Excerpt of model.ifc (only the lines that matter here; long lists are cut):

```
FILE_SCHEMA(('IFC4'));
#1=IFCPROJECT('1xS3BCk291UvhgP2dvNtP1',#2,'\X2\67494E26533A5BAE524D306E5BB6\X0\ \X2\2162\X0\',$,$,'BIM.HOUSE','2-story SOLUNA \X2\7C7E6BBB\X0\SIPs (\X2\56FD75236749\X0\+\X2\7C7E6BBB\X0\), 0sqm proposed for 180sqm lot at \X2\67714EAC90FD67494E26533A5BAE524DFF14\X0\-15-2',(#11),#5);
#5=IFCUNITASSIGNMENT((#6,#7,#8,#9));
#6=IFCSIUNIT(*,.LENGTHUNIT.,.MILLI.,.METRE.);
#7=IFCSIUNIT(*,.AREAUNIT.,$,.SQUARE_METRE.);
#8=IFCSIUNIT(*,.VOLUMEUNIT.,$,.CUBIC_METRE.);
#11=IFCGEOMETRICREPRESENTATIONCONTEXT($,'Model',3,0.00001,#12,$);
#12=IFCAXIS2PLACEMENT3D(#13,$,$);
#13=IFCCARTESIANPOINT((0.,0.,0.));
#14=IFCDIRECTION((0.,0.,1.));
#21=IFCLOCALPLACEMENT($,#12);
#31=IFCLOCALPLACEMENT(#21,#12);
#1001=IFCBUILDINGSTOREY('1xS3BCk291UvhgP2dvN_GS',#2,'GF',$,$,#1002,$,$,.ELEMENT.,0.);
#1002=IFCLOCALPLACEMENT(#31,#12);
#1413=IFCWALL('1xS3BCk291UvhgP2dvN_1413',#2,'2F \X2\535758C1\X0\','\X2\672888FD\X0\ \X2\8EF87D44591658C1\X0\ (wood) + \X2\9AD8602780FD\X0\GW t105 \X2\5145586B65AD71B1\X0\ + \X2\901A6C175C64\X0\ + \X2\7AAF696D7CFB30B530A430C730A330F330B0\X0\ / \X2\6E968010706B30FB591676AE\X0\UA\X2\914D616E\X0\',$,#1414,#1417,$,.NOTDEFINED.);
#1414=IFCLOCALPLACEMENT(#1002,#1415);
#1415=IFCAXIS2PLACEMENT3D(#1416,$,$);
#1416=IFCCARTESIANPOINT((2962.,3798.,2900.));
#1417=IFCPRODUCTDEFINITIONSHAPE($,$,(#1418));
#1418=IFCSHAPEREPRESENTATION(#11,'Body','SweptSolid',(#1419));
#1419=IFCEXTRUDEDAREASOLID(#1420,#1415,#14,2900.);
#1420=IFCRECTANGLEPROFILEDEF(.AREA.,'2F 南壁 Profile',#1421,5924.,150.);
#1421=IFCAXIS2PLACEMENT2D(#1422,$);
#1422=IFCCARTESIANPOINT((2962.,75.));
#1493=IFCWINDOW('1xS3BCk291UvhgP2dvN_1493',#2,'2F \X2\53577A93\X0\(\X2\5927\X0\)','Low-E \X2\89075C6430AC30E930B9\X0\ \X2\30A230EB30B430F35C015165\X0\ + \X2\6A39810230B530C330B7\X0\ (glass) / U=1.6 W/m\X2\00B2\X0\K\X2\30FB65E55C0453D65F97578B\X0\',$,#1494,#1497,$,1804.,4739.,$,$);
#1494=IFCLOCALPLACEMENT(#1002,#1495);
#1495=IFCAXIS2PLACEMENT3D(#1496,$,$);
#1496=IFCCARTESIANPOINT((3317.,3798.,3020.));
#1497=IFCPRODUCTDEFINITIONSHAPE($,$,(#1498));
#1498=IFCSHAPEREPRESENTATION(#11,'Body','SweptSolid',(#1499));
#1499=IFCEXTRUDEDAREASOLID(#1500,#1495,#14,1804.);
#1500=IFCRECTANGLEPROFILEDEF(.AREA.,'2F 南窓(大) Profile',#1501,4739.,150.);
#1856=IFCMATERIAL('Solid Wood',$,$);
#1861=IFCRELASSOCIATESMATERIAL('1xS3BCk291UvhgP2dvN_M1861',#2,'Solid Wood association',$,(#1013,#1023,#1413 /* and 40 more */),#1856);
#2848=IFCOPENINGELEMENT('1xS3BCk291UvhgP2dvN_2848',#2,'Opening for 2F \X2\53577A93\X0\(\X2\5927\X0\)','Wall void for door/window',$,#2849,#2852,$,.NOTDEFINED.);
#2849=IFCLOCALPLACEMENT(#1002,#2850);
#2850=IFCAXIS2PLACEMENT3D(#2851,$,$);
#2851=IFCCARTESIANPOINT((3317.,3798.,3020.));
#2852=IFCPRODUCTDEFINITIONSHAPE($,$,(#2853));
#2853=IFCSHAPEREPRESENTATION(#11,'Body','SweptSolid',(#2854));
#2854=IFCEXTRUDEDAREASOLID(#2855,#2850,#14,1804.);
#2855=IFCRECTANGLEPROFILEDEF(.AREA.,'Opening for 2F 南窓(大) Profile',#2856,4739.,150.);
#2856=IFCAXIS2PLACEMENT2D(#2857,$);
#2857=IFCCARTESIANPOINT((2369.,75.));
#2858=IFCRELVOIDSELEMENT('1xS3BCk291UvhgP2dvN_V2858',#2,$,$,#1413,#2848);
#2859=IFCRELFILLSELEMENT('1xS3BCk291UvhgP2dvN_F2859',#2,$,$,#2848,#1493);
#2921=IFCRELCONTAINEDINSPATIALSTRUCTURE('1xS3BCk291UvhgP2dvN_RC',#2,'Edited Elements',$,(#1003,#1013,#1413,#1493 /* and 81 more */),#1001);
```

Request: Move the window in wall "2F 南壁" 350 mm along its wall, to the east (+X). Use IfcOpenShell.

```python
import ifcopenshell
import ifcopenshell.api.geometry
import ifcopenshell.util.placement
import ifcopenshell.util.unit

model = ifcopenshell.open("model.ifc")
unit_scale = ifcopenshell.util.unit.calculate_unit_scale(model)

window = model.by_guid("1xS3BCk291UvhgP2dvN_1493")
opening = window.FillsVoids[0].RelatingOpeningElement
wall = opening.VoidsElements[0].RelatingBuildingElement

wall_matrix = ifcopenshell.util.placement.get_local_placement(wall.ObjectPlacement)
shift = wall_matrix[:3, 0] * 0.35 / unit_scale
before = ifcopenshell.util.placement.get_local_placement(window.ObjectPlacement)[:3, 3].copy()

# The window is not placed relative to its opening, so move both.
for product in (opening, window):
    matrix = ifcopenshell.util.placement.get_local_placement(product.ObjectPlacement)
    matrix[:3, 3] += shift
    ifcopenshell.api.geometry.edit_object_placement(model, product=product, matrix=matrix, is_si=False)

after = ifcopenshell.util.placement.get_local_placement(window.ObjectPlacement)[:3, 3]
print("window moved by", (after - before).round(3) + 0.0)

model.write("model_edited.ifc")
```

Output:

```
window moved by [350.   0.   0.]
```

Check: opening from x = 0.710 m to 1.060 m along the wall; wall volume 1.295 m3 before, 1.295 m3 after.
